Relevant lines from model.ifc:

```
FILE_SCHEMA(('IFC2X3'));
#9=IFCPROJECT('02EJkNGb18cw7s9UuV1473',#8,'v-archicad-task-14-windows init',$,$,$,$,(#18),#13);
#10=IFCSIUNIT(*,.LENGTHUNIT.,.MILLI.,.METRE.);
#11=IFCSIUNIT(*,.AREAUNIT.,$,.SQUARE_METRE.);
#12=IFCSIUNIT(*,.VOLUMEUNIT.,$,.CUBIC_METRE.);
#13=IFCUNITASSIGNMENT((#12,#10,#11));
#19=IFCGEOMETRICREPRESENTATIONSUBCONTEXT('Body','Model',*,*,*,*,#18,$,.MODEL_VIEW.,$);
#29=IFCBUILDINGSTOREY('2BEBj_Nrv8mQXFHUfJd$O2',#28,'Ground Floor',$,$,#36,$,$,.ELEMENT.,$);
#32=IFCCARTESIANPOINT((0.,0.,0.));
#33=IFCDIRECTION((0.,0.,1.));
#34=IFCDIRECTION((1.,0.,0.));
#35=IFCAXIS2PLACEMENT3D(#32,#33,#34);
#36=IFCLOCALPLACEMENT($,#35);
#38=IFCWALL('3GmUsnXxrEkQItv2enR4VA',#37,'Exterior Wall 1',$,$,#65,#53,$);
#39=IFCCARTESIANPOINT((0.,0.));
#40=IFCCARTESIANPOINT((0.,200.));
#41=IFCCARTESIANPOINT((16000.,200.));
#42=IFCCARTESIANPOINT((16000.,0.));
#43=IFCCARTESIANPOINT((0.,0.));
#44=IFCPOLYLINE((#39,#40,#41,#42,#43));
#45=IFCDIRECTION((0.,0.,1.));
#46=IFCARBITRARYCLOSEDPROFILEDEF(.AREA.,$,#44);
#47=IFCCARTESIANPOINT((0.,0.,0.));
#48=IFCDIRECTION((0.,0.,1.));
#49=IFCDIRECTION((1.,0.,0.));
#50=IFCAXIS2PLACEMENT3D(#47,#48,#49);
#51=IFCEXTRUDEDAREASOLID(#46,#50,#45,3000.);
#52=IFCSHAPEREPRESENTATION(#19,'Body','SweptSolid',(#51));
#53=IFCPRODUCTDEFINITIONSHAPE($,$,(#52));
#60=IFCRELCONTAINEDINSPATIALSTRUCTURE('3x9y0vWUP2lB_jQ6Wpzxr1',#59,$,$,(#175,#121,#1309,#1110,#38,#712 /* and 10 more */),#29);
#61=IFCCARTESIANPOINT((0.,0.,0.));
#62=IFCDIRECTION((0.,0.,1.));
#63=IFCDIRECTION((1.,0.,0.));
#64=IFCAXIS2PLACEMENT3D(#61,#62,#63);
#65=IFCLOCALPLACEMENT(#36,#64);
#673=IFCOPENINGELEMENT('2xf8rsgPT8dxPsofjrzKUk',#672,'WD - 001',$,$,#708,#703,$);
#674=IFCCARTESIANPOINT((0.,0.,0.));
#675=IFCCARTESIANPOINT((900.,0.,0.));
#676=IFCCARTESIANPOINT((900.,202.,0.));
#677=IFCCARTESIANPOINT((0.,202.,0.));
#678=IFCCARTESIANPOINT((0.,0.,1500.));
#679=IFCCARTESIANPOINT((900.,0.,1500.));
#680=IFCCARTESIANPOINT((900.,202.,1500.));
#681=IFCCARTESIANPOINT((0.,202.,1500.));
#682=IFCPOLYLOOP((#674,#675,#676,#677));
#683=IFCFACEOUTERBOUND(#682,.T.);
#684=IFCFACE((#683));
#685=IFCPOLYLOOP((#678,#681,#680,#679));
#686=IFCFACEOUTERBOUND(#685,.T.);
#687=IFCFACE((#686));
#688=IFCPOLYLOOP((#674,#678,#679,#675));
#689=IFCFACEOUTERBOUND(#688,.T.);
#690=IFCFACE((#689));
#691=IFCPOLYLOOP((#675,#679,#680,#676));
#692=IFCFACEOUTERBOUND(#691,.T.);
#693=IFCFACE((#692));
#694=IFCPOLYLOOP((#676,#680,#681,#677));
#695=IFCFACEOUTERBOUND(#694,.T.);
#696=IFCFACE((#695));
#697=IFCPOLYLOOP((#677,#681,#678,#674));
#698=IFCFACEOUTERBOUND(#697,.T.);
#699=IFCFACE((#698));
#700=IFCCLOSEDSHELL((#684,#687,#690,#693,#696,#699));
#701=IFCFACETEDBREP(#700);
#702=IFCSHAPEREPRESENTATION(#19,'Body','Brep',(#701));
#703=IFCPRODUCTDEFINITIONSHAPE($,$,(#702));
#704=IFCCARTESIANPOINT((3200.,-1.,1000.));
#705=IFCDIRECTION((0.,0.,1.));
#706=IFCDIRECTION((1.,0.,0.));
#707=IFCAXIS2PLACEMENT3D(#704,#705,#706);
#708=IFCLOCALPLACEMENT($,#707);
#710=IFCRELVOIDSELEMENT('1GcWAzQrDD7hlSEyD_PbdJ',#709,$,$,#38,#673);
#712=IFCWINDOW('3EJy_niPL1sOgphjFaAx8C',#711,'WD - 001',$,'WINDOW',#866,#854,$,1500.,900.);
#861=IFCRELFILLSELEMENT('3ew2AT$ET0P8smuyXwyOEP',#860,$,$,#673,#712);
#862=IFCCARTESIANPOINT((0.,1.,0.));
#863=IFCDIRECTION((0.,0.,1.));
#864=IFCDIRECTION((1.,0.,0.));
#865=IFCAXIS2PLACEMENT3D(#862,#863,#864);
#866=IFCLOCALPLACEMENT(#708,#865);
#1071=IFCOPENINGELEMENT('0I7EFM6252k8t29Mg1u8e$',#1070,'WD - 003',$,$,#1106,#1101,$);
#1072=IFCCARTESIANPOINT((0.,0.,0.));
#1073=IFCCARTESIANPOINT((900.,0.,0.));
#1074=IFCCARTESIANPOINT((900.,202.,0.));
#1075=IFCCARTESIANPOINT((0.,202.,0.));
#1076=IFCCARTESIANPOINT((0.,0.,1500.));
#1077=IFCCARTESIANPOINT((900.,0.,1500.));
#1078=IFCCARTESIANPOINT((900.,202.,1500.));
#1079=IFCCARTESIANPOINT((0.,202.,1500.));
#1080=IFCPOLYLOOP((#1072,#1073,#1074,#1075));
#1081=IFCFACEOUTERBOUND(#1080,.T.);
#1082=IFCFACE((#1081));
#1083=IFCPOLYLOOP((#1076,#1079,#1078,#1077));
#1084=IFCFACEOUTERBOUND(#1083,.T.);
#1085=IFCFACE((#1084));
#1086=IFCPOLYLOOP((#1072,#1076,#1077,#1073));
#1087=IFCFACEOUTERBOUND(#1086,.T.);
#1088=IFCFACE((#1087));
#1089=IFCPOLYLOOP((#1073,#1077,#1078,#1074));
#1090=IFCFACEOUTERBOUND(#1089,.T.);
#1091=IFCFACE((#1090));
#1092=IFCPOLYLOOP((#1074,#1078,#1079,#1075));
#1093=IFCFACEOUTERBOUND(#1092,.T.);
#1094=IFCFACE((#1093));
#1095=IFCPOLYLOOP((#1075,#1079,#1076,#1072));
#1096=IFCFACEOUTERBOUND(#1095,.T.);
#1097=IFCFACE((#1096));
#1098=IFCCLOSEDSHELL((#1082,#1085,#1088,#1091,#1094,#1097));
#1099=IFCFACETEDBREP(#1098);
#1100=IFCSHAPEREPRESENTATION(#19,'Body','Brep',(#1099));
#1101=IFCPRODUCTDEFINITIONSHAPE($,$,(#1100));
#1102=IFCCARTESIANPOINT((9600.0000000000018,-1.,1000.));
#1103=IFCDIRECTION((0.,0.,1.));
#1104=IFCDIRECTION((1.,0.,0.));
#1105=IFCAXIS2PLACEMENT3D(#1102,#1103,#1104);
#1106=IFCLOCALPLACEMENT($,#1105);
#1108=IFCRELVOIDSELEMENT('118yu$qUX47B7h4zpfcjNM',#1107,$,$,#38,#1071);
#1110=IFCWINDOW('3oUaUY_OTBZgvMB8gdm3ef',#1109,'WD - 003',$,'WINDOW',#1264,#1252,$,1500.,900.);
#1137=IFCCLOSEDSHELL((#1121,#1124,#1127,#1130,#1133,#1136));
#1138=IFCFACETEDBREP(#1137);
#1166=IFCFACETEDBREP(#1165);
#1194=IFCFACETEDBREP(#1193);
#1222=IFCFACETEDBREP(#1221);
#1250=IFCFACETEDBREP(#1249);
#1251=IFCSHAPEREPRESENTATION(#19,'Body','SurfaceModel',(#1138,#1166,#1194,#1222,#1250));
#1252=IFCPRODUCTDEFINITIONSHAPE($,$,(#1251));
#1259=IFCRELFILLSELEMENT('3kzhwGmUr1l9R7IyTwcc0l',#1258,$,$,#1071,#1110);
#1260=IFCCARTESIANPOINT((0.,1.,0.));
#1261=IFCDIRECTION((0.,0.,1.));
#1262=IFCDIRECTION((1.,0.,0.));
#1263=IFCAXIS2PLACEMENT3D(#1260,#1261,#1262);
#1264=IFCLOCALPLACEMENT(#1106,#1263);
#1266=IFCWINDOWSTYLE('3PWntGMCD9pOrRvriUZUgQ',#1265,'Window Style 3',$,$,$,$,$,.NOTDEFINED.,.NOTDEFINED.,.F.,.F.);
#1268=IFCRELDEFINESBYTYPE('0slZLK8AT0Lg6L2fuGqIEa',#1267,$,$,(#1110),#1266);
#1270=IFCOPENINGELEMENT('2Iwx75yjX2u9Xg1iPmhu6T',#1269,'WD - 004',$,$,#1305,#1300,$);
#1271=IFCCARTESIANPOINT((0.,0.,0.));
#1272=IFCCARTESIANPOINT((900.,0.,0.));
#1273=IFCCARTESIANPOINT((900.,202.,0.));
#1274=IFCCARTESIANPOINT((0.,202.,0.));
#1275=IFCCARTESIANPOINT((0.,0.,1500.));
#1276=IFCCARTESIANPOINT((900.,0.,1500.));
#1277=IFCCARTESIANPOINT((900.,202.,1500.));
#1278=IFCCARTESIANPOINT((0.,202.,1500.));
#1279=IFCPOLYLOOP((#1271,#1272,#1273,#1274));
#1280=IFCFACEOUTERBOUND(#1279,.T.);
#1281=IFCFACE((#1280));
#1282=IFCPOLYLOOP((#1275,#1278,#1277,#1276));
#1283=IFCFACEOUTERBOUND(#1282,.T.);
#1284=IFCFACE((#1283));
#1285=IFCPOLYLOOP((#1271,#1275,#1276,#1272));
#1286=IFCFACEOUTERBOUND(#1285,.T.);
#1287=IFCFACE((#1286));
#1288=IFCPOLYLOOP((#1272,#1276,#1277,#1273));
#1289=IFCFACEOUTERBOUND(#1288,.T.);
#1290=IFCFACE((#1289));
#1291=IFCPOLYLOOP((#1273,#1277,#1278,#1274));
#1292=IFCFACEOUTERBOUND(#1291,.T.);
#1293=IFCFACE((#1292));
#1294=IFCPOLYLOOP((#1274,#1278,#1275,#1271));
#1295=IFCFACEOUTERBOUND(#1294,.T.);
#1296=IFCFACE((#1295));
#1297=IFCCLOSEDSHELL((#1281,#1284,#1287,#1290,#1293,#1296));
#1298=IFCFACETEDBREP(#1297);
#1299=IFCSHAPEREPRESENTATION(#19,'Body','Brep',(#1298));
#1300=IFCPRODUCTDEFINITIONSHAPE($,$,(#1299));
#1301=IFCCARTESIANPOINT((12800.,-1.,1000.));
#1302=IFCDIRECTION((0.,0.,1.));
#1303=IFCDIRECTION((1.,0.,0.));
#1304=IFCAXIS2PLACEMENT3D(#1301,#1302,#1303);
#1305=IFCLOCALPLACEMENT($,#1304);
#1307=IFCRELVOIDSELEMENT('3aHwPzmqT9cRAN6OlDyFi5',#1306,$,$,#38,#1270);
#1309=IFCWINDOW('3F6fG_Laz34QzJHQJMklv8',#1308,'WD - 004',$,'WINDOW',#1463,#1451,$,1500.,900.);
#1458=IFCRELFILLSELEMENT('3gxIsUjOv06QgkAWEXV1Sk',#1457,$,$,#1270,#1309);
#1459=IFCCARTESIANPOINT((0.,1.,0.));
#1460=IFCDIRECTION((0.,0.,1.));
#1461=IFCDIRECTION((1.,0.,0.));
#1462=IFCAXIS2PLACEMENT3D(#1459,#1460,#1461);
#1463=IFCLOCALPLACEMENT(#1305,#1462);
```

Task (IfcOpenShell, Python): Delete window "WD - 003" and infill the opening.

```python
import ifcopenshell
import ifcopenshell.api.feature
import ifcopenshell.api.root
import ifcopenshell.geom
import ifcopenshell.util.shape

model = ifcopenshell.open("model.ifc")
settings = ifcopenshell.geom.settings()


def volume(element):
    """Net volume in cubic metres, openings subtracted."""
    shape = ifcopenshell.geom.create_shape(settings, element)
    return ifcopenshell.util.shape.get_volume(shape.geometry)


window = model.by_id(1110)
opening = window.FillsVoids[0].RelatingOpeningElement
wall = opening.VoidsElements[0].RelatingBuildingElement
before = volume(wall)

ifcopenshell.api.root.remove_product(model, product=window)
ifcopenshell.api.feature.remove_feature(model, feature=opening)

after = volume(wall)

print(f"wall volume {before:.3f} -> {after:.3f} m3")

model.write("model_edited.ifc")
```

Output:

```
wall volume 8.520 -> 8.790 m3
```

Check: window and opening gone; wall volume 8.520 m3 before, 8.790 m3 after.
